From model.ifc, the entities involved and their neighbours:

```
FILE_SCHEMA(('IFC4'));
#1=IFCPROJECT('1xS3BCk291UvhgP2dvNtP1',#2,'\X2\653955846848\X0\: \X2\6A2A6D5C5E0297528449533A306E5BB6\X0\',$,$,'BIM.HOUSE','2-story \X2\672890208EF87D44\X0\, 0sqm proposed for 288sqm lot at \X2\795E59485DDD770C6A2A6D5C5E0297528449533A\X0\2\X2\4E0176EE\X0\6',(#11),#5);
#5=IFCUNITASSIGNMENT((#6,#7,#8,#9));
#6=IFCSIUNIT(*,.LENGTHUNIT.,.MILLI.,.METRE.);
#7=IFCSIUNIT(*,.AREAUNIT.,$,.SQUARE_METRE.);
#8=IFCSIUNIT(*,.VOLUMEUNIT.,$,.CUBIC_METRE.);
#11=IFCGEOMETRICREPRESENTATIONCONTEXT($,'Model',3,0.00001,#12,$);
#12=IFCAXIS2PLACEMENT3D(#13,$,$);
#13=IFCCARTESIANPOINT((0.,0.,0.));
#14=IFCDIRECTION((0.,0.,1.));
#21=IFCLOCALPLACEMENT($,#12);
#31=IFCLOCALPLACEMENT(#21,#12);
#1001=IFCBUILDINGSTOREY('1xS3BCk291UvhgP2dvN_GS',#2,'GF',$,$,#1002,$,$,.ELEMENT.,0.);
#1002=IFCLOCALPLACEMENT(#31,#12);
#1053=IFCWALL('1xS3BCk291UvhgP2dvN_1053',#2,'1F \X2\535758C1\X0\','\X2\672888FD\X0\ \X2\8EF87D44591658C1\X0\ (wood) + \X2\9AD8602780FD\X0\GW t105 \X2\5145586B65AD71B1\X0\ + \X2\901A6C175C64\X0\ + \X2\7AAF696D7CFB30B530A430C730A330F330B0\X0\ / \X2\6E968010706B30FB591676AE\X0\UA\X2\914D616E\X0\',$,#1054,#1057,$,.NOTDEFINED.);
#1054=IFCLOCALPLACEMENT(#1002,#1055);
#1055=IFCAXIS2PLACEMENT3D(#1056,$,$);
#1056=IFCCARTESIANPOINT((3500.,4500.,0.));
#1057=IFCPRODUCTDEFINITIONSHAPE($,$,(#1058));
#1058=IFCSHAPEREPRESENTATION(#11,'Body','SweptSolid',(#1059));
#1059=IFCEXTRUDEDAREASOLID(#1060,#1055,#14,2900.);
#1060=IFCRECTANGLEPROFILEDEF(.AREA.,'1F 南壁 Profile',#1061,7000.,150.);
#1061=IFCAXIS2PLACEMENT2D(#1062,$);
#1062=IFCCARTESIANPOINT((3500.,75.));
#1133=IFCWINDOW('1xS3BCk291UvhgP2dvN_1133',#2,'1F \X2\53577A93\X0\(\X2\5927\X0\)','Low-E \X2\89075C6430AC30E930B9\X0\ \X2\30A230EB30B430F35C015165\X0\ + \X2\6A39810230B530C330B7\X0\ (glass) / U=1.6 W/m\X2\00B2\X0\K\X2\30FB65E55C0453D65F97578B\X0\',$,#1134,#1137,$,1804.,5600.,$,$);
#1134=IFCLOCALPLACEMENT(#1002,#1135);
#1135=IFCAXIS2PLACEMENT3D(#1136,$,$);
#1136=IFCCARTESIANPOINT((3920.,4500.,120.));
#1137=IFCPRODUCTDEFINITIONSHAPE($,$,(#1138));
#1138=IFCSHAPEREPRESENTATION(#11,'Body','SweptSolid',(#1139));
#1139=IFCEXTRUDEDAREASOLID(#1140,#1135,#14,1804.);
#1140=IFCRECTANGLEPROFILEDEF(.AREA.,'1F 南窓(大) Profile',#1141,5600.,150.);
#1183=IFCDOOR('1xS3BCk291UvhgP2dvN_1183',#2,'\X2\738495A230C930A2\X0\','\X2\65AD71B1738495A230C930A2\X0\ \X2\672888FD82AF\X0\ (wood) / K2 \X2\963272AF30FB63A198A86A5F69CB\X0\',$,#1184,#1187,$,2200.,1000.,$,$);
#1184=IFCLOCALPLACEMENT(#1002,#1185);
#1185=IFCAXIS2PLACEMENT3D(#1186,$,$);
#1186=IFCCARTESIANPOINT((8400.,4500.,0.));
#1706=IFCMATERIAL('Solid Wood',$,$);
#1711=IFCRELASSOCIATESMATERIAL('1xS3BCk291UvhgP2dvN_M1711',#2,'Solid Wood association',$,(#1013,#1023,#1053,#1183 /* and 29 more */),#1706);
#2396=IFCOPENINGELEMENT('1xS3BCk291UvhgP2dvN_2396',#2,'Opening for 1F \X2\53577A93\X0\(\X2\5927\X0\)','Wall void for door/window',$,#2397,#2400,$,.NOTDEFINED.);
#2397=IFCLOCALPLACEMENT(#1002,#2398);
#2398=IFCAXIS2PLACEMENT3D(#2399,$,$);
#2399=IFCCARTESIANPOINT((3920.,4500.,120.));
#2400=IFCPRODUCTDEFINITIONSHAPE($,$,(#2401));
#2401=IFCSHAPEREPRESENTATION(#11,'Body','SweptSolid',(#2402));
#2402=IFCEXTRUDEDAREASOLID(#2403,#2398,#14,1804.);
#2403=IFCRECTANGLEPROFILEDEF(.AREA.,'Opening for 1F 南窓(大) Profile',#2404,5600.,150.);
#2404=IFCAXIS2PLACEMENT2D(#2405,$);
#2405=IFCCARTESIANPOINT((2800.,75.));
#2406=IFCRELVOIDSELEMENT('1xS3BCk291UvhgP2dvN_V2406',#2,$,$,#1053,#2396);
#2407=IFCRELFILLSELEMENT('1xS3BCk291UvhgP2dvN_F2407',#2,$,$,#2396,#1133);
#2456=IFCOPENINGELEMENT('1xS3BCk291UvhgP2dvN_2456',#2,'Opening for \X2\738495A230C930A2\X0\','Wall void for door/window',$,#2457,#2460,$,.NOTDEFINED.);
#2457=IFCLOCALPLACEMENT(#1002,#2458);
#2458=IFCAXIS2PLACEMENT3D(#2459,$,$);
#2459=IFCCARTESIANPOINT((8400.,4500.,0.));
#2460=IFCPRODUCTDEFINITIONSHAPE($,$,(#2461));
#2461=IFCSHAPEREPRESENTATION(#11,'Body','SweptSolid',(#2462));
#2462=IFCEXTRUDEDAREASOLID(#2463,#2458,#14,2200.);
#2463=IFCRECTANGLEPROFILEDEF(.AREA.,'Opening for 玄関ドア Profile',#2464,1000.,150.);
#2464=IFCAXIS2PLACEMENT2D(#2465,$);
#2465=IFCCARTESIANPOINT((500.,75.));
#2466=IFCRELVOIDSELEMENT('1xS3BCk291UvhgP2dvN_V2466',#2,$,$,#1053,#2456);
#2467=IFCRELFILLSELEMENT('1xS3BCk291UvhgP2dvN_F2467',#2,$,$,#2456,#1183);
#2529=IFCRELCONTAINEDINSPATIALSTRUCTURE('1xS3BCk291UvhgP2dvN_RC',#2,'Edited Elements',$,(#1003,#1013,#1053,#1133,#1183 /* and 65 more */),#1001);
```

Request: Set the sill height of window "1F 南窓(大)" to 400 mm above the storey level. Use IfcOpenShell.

```python
import numpy as np
import ifcopenshell
import ifcopenshell.api.geometry
import ifcopenshell.geom
import ifcopenshell.util.element
import ifcopenshell.util.placement
import ifcopenshell.util.shape
import ifcopenshell.util.unit

model = ifcopenshell.open("model.ifc")
unit_scale = ifcopenshell.util.unit.calculate_unit_scale(model)

window = model.by_guid("1xS3BCk291UvhgP2dvN_1133")
opening = window.FillsVoids[0].RelatingOpeningElement
storey = ifcopenshell.util.element.get_container(window, ifc_class="IfcBuildingStorey")
level = ifcopenshell.util.placement.get_local_placement(storey.ObjectPlacement)[2, 3]

# The opening's origin need not be at the sill, so measure its lowest point.
shape = ifcopenshell.geom.create_shape(ifcopenshell.geom.settings(), opening)
bottom = ifcopenshell.util.shape.get_shape_bottom_elevation(shape, shape.geometry) / unit_scale
dz = level + 0.4 / unit_scale - bottom

shift = np.array([0.0, 0.0, dz])
# The window is not placed relative to its opening, so move both.
for product in (opening, window):
    matrix = ifcopenshell.util.placement.get_local_placement(product.ObjectPlacement)
    matrix[:3, 3] += shift
    ifcopenshell.api.geometry.edit_object_placement(model, product=product, matrix=matrix, is_si=False)

print(f"moved by {dz * unit_scale:+.3f} m")

model.write("model-out.ifc")
```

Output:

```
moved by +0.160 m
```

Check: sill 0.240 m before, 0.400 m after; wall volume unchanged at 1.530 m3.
